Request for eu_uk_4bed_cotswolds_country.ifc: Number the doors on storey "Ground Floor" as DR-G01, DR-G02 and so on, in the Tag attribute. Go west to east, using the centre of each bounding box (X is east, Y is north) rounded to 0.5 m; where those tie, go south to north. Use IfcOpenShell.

First a look at what the model holds.

```python
import ifcopenshell
import ifcopenshell.util.element
import ifcopenshell.util.placement

model = ifcopenshell.open("eu_uk_4bed_cotswolds_country.ifc")
print(model.schema)
storey = next(s for s in model.by_type("IfcBuildingStorey") if s.Name == "Ground Floor")
doors = [e for e in ifcopenshell.util.element.get_decomposition(storey) if e.is_a("IfcDoor")]
for e in sorted(doors, key=lambda e: e.id()):
    origin = ifcopenshell.util.placement.get_local_placement(e.ObjectPlacement)[:3, 3]
    print(e.id(), e.Tag, e.Name, origin.round(2) + 0.0, sep=" | ")
```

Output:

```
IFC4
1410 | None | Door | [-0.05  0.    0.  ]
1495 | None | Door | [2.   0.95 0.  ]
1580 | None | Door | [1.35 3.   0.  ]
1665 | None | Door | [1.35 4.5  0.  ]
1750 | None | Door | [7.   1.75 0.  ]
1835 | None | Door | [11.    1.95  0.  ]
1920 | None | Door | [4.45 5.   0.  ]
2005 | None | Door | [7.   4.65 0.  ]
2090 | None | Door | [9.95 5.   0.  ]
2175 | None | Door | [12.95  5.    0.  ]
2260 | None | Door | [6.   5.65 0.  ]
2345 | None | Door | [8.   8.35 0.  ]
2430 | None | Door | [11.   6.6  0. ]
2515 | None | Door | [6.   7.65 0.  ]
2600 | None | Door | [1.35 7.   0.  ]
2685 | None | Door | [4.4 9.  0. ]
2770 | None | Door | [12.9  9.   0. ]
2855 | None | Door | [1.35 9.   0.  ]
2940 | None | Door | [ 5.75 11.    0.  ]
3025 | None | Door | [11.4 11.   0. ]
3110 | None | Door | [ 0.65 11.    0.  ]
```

```python
import ifcopenshell
import ifcopenshell.geom
import ifcopenshell.util.element
import ifcopenshell.util.shape

model = ifcopenshell.open("eu_uk_4bed_cotswolds_country.ifc")
settings = ifcopenshell.geom.settings()
settings.set("use-world-coords", True)


def centre(element):
    shape = ifcopenshell.geom.create_shape(settings, element)
    return ifcopenshell.util.shape.get_bbox_centroid(shape.geometry)


storey = next(s for s in model.by_type("IfcBuildingStorey") if s.Name == "Ground Floor")
doors = [e for e in ifcopenshell.util.element.get_decomposition(storey) if e.is_a("IfcDoor")]

# Insertion points can sit at a corner or the storey origin, so sort by the geometry (in metres).
centres = {e: centre(e) for e in doors}
doors.sort(key=lambda e: (round(centres[e][0] / 0.5), centres[e][1]))

for i, e in enumerate(doors, start=1):
    number = f"DR-G{i:02d}"
    e.Tag = number
    print(e.id(), number)

model.write("eu_uk_4bed_cotswolds_country_edited.ifc")
```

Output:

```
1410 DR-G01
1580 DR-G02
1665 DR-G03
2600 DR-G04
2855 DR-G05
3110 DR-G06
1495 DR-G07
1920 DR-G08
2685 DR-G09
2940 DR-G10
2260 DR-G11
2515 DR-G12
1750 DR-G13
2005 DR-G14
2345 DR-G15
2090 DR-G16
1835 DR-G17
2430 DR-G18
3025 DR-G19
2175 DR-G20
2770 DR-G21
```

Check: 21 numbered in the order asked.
